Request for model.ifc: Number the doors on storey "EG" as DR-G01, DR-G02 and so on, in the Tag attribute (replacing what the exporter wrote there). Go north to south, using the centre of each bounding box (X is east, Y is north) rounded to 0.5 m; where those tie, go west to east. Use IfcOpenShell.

First a look at what the model holds.

```python
import ifcopenshell
import ifcopenshell.util.element
import ifcopenshell.util.placement

model = ifcopenshell.open("model.ifc")
print(model.schema)
storey = next(s for s in model.by_type("IfcBuildingStorey") if s.Name == "EG")
doors = [e for e in ifcopenshell.util.element.get_decomposition(storey) if e.is_a("IfcDoor")]
for e in sorted(doors, key=lambda e: e.id()):
    origin = ifcopenshell.util.placement.get_local_placement(e.ObjectPlacement)[:3, 3]
    print(e.id(), e.Tag, e.Name, origin.round(2) + 0.0, sep=" | ")
```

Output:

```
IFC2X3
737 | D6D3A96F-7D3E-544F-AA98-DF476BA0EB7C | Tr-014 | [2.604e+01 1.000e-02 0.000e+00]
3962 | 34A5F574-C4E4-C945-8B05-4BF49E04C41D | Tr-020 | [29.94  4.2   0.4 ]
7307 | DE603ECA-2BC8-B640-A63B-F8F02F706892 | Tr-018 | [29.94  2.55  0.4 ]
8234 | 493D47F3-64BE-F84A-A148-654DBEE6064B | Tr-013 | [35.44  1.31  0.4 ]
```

```python
import ifcopenshell
import ifcopenshell.geom
import ifcopenshell.util.element
import ifcopenshell.util.shape

model = ifcopenshell.open("model.ifc")
settings = ifcopenshell.geom.settings()
settings.set("use-world-coords", True)


def centre(element):
    shape = ifcopenshell.geom.create_shape(settings, element)
    return ifcopenshell.util.shape.get_bbox_centroid(shape.geometry)


storey = next(s for s in model.by_type("IfcBuildingStorey") if s.Name == "EG")
doors = [e for e in ifcopenshell.util.element.get_decomposition(storey) if e.is_a("IfcDoor")]

# Insertion points can sit at a corner or the storey origin, so sort by the geometry (in metres).
centres = {e: centre(e) for e in doors}
doors.sort(key=lambda e: (-round(centres[e][1] / 0.5), centres[e][0]))

for i, e in enumerate(doors, start=1):
    number = f"DR-G{i:02d}"
    e.Tag = number
    print(e.id(), number)

model.write("model_v2.ifc")
```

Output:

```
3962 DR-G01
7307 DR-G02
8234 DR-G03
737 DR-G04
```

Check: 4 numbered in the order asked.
